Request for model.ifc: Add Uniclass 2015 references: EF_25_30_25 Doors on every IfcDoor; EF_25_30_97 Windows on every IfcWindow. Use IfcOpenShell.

First a look at what the model holds.

```python
import ifcopenshell

model = ifcopenshell.open("model.ifc")
print(model.schema)
print("classifications:", [c.Name for c in model.by_type("IfcClassification")])
for ifc_class in ("IfcDoor", "IfcRoof", "IfcStair", "IfcWall", "IfcWindow"):
    print(ifc_class, len(model.by_type(ifc_class)))
```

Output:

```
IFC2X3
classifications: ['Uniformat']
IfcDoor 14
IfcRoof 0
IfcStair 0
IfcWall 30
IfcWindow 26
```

```python
import ifcopenshell
import ifcopenshell.api.classification

model = ifcopenshell.open("model.ifc")

# IFC2X3 requires Source and Edition and has no link from the project to the system.
system = model.create_entity("IfcClassification", Source="NBS", Edition="2015", Name="Uniclass 2015")

codes = {
    "IfcDoor": ("EF_25_30_25", "Doors"),
    "IfcWindow": ("EF_25_30_97", "Windows"),
}
for ifc_class, (code, name) in codes.items():
    products = model.by_type(ifc_class)
    ifcopenshell.api.classification.add_reference(
        model, products=products, classification=system, identification=code, name=name
    )
    print(code, len(products))

model.write("model-out.ifc")
```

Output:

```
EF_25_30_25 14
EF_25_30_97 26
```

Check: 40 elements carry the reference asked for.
